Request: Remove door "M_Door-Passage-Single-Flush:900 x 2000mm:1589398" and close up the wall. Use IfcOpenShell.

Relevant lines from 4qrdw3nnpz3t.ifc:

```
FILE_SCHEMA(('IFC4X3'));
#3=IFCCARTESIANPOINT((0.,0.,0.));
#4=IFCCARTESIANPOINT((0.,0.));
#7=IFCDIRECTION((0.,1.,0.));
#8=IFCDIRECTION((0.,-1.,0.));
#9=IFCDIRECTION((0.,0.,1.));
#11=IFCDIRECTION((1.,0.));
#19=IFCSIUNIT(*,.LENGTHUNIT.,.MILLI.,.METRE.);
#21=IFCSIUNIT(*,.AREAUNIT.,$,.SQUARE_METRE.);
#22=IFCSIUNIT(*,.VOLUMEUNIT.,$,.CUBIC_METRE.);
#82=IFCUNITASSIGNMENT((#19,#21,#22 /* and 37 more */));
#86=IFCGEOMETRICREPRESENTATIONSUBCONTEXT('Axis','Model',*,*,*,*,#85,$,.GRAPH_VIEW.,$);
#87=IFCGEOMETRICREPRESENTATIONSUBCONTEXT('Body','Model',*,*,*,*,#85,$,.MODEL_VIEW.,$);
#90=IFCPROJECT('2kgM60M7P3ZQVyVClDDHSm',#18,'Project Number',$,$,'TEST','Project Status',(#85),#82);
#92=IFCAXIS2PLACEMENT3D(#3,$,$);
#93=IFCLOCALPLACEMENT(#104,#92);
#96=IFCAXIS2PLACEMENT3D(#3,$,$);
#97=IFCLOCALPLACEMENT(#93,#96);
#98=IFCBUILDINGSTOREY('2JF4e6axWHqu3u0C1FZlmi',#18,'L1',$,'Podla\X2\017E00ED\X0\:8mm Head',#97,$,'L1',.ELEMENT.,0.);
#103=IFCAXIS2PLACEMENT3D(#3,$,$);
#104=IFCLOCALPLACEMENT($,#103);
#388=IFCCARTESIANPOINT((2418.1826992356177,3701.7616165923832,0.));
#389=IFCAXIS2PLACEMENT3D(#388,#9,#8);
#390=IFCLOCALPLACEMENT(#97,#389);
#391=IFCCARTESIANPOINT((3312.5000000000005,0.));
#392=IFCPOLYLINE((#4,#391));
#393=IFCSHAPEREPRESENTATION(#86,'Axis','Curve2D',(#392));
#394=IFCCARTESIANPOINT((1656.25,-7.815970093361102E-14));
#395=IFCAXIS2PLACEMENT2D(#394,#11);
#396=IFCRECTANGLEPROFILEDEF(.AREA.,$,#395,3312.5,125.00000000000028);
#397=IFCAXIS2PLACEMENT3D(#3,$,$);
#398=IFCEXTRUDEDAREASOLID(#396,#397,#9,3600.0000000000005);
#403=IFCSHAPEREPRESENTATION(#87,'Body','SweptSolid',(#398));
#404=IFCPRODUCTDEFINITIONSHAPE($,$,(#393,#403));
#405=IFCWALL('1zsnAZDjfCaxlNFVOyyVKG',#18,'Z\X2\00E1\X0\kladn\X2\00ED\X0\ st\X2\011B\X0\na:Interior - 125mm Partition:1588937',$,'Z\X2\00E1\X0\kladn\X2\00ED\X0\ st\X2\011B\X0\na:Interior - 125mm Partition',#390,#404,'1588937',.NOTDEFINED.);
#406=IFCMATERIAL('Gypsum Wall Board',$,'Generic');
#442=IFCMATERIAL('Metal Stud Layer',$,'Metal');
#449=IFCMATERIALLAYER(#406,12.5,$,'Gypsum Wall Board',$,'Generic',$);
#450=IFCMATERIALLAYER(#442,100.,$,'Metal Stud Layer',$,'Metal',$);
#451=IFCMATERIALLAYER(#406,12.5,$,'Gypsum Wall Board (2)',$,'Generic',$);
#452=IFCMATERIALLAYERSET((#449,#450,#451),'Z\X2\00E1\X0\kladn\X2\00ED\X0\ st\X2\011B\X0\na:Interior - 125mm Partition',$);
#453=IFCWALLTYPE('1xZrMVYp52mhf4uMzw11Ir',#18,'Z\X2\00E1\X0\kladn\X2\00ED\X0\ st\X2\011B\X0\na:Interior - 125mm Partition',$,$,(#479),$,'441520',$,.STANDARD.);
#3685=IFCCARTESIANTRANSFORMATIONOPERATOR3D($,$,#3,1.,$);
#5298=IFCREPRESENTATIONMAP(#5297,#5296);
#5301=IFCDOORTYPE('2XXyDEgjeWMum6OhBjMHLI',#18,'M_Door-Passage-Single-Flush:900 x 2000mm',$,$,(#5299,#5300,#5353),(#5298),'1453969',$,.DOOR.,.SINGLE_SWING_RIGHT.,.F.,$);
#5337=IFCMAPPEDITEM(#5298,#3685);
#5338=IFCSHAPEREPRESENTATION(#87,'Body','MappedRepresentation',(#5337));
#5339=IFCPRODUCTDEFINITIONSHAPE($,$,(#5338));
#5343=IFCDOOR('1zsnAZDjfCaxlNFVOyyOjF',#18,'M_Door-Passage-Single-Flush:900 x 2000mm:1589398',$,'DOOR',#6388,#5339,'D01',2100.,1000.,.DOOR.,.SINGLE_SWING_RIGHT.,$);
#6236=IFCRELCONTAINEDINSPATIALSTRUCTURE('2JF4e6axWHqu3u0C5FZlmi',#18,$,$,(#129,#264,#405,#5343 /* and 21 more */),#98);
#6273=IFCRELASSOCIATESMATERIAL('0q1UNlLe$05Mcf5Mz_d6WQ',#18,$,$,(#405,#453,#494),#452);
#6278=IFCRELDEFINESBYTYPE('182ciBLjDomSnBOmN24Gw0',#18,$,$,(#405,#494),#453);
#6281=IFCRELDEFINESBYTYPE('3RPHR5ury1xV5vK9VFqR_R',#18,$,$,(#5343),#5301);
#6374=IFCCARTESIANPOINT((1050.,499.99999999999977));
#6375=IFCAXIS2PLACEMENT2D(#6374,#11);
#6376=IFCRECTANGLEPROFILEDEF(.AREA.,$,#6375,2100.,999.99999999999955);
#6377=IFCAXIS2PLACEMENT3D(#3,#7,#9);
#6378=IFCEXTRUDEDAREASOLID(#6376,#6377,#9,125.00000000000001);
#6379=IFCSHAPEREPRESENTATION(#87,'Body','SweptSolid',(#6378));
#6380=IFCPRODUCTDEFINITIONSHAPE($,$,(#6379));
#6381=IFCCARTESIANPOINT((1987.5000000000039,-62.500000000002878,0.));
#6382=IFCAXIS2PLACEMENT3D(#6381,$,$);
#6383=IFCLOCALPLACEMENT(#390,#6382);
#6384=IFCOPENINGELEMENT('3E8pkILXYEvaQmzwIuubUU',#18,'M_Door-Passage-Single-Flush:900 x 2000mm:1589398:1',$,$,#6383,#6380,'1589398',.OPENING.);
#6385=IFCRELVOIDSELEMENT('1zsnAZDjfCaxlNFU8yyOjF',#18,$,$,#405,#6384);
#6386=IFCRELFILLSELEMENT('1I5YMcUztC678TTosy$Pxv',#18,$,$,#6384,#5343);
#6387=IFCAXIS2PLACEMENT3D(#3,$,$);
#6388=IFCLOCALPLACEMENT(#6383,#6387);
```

```python
import ifcopenshell
import ifcopenshell.api.feature
import ifcopenshell.api.root
import ifcopenshell.geom
import ifcopenshell.util.shape

model = ifcopenshell.open("4qrdw3nnpz3t.ifc")
settings = ifcopenshell.geom.settings()


def volume(element):
    """Net volume in cubic metres, openings subtracted."""
    shape = ifcopenshell.geom.create_shape(settings, element)
    return ifcopenshell.util.shape.get_volume(shape.geometry)


door = model.by_guid("1zsnAZDjfCaxlNFVOyyOjF")
opening = door.FillsVoids[0].RelatingOpeningElement
wall = opening.VoidsElements[0].RelatingBuildingElement
before = volume(wall)

ifcopenshell.api.root.remove_product(model, product=door)
ifcopenshell.api.feature.remove_feature(model, feature=opening)

after = volume(wall)

print(f"wall volume {before:.3f} -> {after:.3f} m3")

model.write("4qrdw3nnpz3t_rev.ifc")
```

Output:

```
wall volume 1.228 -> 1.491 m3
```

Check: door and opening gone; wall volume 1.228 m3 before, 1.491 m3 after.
